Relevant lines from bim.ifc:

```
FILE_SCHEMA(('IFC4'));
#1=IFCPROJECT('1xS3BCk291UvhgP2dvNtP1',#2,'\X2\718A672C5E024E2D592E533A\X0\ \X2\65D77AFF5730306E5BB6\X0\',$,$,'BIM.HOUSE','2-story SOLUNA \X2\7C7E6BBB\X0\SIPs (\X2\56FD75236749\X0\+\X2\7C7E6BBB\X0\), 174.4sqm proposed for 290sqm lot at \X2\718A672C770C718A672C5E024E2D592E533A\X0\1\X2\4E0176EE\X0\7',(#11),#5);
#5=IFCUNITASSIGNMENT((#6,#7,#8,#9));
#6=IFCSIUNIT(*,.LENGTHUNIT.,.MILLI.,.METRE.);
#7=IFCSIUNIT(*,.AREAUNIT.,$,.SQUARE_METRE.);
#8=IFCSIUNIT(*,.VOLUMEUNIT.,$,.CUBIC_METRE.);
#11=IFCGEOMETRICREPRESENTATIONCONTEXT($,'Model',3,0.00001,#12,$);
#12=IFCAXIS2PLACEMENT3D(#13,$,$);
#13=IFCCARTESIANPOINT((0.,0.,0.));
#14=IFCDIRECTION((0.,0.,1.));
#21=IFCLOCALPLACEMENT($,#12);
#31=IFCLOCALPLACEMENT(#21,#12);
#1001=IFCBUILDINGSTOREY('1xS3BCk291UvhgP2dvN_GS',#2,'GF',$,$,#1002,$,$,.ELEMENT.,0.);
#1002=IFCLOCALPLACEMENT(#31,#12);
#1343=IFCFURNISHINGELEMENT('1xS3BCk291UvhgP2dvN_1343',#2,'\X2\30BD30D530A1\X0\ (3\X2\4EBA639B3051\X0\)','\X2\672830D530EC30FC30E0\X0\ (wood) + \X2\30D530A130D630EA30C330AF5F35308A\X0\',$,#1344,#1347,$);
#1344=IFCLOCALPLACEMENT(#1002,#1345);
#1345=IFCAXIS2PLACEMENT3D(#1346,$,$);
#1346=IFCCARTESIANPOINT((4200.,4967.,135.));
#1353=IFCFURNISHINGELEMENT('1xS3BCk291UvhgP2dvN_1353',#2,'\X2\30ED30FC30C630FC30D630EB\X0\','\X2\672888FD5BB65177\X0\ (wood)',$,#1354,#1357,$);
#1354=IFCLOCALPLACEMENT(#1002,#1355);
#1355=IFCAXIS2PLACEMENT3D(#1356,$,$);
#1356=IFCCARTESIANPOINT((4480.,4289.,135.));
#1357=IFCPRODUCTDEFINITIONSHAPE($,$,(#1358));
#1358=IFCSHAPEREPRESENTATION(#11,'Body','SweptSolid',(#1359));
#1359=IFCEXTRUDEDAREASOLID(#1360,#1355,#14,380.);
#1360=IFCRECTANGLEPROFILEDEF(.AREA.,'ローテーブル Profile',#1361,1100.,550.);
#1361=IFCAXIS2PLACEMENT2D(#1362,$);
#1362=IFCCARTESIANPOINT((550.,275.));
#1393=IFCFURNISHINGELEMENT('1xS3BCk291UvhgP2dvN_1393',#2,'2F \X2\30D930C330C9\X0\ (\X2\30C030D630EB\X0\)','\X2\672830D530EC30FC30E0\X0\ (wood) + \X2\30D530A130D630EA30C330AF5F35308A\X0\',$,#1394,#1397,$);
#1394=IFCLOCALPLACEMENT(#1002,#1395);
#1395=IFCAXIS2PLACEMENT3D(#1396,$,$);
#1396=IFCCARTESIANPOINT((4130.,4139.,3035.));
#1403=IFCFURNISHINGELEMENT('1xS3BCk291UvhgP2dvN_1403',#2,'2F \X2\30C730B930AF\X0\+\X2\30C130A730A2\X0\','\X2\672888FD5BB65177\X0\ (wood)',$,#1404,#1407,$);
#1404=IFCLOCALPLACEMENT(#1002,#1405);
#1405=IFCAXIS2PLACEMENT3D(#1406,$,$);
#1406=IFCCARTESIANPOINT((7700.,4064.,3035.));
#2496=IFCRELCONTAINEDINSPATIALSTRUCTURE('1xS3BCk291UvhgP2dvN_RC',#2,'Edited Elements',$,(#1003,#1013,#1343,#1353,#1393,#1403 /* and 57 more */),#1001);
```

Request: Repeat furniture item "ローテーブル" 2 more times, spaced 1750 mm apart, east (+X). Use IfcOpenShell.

```python
import numpy as np
import ifcopenshell
import ifcopenshell.api.geometry
import ifcopenshell.api.root
import ifcopenshell.util.element
import ifcopenshell.util.placement

model = ifcopenshell.open("bim.ifc")


def reuse_history(source, copy):
    """copy_class also copies each property set's owner history, people and application; keep the originals."""
    for rel in copy.IsDefinedBy:
        if rel.is_a("IfcRelDefinesByProperties") and (history := rel.RelatingPropertyDefinition.OwnerHistory):
            rel.RelatingPropertyDefinition.OwnerHistory = source.OwnerHistory
            ifcopenshell.util.element.remove_deep2(model, history)


source = model.by_guid("1xS3BCk291UvhgP2dvN_1353")
base = ifcopenshell.util.placement.get_local_placement(source.ObjectPlacement)
step = np.array([1.0, 0.0, 0.0]) * 1750.0

for i in range(1, 3):
    copy = ifcopenshell.api.root.copy_class(model, product=source)
    copy.Representation = ifcopenshell.util.element.copy_deep(
        model, source.Representation, exclude=["IfcGeometricRepresentationContext", "IfcRepresentationMap"]
    )
    reuse_history(source, copy)
    matrix = base.copy()
    matrix[:3, 3] += i * step
    print("added at", matrix[:3, 3].round(3) + 0.0)
    ifcopenshell.api.geometry.edit_object_placement(model, product=copy, matrix=matrix, is_si=False)

model.write("bim_edited.ifc")
```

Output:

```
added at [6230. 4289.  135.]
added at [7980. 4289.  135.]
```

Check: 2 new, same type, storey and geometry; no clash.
